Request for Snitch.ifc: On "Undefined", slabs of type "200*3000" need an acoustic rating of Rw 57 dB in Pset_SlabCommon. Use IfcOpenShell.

First a look at what the model holds.

```python
import ifcopenshell
import ifcopenshell.util.element

model = ifcopenshell.open("Snitch.ifc")
print(model.schema)
storey = next(s for s in model.by_type("IfcBuildingStorey") if s.Name == "Undefined")
slabs = [e for e in ifcopenshell.util.element.get_decomposition(storey) if e.is_a("IfcSlab")]
seen = {}
for e in slabs:
    element_type = ifcopenshell.util.element.get_type(e)
    key = (element_type.Name if element_type != e and element_type else None, ifcopenshell.util.element.get_pset(e, "Pset_SlabCommon", "AcousticRating"))
    seen[key] = seen.get(key, 0) + 1
for (name, value), count in sorted(seen.items(), key=str):
    print(count, "x", name, "|", value)
```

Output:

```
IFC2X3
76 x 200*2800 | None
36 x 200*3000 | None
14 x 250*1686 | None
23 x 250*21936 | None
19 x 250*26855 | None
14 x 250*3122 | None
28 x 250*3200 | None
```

```python
import ifcopenshell
import ifcopenshell.api.pset
import ifcopenshell.util.element

model = ifcopenshell.open("Snitch.ifc")

storey = next(s for s in model.by_type("IfcBuildingStorey") if s.Name == "Undefined")
slabs = [e for e in ifcopenshell.util.element.get_decomposition(storey) if e.is_a("IfcSlab")]

count = 0
for e in slabs:
    element_type = ifcopenshell.util.element.get_type(e)
    if element_type in (None, e) or element_type.Name != "200*3000":
        continue
    found = ifcopenshell.util.element.get_pset(e, "Pset_SlabCommon", should_inherit=False)
    if found:
        pset = model.by_id(found["id"])
        if len(ifcopenshell.util.element.get_elements_by_pset(pset)) > 1:
            pset = ifcopenshell.api.pset.unshare_pset(model, products=[e], pset=pset)[0]
    else:
        pset = ifcopenshell.api.pset.add_pset(model, product=e, name="Pset_SlabCommon")
    ifcopenshell.api.pset.edit_pset(model, pset=pset, properties={"AcousticRating": "Rw 57 dB"})
    count += 1

print(count, "slabs updated")

model.write("Snitch-out.ifc")
```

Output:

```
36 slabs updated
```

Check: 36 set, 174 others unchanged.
